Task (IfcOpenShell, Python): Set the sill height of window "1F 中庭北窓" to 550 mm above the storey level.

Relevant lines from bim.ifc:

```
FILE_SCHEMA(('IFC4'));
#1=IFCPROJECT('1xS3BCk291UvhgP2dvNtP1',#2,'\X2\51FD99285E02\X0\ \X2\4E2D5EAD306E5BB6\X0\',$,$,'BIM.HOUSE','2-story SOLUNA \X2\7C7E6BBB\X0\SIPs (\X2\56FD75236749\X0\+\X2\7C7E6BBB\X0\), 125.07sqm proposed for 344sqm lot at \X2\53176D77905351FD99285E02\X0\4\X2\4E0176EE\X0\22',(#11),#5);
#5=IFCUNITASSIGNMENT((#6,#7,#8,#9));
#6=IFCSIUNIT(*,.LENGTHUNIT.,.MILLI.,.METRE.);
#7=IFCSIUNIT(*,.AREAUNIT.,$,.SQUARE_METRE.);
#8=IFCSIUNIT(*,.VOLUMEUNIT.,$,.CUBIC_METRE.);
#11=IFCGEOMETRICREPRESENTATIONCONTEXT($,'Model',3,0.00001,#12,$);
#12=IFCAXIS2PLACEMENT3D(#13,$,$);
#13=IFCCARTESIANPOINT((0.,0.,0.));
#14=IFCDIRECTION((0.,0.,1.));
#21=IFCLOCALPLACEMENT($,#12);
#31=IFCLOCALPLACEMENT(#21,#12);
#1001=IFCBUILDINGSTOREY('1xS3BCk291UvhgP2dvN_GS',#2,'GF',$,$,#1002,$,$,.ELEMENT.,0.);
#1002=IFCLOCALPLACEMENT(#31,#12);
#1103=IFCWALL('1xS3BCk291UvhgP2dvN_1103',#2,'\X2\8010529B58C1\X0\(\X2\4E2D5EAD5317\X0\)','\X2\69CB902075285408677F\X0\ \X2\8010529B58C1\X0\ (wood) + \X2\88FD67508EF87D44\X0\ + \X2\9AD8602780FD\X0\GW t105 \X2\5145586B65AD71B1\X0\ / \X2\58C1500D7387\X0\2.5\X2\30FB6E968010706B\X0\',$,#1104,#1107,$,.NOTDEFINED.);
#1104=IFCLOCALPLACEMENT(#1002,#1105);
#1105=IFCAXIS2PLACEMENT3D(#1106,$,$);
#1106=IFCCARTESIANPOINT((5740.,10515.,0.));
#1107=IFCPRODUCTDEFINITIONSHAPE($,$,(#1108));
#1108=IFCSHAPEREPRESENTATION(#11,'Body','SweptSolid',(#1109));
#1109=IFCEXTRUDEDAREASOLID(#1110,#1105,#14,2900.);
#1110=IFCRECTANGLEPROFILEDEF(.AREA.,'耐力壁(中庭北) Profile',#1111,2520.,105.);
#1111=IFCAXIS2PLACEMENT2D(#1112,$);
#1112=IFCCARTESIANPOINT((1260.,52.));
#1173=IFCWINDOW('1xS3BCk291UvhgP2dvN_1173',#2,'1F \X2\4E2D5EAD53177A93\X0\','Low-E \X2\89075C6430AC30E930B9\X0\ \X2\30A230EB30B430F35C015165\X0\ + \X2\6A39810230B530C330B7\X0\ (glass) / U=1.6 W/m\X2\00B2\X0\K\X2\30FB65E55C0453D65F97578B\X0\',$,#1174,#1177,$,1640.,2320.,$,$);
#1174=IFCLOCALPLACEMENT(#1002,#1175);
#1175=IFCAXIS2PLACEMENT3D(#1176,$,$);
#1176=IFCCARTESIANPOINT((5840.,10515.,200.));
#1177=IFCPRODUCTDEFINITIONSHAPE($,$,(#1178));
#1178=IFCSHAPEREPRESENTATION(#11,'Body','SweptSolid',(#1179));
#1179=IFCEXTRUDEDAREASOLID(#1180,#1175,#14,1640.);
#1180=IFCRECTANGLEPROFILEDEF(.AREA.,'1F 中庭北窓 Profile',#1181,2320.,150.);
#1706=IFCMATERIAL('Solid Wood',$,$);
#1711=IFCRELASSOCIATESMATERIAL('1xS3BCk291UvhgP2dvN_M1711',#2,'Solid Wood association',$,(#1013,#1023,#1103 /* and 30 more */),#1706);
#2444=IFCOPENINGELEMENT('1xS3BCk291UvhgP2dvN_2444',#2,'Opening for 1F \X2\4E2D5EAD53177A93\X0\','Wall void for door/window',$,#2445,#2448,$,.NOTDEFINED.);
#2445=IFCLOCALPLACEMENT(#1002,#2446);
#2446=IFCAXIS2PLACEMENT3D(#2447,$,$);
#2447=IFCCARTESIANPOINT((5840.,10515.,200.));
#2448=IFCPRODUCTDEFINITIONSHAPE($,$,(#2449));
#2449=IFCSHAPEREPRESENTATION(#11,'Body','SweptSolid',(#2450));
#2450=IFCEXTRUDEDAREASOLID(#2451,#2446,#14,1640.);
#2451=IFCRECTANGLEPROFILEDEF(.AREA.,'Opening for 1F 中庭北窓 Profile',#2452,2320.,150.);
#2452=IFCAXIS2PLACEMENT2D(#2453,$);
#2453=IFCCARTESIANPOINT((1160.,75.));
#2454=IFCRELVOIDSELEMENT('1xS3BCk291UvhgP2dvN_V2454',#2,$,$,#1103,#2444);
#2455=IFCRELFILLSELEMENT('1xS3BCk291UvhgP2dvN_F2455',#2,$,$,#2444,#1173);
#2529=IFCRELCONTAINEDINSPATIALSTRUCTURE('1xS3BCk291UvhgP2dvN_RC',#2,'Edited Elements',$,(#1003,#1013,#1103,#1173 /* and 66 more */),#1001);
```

```python
import numpy as np
import ifcopenshell
import ifcopenshell.api.geometry
import ifcopenshell.geom
import ifcopenshell.util.element
import ifcopenshell.util.placement
import ifcopenshell.util.shape
import ifcopenshell.util.unit

model = ifcopenshell.open("bim.ifc")
unit_scale = ifcopenshell.util.unit.calculate_unit_scale(model)

window = model.by_guid("1xS3BCk291UvhgP2dvN_1173")
opening = window.FillsVoids[0].RelatingOpeningElement
storey = ifcopenshell.util.element.get_container(window, ifc_class="IfcBuildingStorey")
level = ifcopenshell.util.placement.get_local_placement(storey.ObjectPlacement)[2, 3]

# The opening's origin need not be at the sill, so measure its lowest point.
shape = ifcopenshell.geom.create_shape(ifcopenshell.geom.settings(), opening)
bottom = ifcopenshell.util.shape.get_shape_bottom_elevation(shape, shape.geometry) / unit_scale
dz = level + 550.0 - bottom

shift = np.array([0.0, 0.0, dz])
# The window is not placed relative to its opening, so move both.
for product in (opening, window):
    matrix = ifcopenshell.util.placement.get_local_placement(product.ObjectPlacement)
    matrix[:3, 3] += shift
    ifcopenshell.api.geometry.edit_object_placement(model, product=product, matrix=matrix, is_si=False)

print(f"moved by {dz * unit_scale:+.3f} m")

model.write("bim-out.ifc")
```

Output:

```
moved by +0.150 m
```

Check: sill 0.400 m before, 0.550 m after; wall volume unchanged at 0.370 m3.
